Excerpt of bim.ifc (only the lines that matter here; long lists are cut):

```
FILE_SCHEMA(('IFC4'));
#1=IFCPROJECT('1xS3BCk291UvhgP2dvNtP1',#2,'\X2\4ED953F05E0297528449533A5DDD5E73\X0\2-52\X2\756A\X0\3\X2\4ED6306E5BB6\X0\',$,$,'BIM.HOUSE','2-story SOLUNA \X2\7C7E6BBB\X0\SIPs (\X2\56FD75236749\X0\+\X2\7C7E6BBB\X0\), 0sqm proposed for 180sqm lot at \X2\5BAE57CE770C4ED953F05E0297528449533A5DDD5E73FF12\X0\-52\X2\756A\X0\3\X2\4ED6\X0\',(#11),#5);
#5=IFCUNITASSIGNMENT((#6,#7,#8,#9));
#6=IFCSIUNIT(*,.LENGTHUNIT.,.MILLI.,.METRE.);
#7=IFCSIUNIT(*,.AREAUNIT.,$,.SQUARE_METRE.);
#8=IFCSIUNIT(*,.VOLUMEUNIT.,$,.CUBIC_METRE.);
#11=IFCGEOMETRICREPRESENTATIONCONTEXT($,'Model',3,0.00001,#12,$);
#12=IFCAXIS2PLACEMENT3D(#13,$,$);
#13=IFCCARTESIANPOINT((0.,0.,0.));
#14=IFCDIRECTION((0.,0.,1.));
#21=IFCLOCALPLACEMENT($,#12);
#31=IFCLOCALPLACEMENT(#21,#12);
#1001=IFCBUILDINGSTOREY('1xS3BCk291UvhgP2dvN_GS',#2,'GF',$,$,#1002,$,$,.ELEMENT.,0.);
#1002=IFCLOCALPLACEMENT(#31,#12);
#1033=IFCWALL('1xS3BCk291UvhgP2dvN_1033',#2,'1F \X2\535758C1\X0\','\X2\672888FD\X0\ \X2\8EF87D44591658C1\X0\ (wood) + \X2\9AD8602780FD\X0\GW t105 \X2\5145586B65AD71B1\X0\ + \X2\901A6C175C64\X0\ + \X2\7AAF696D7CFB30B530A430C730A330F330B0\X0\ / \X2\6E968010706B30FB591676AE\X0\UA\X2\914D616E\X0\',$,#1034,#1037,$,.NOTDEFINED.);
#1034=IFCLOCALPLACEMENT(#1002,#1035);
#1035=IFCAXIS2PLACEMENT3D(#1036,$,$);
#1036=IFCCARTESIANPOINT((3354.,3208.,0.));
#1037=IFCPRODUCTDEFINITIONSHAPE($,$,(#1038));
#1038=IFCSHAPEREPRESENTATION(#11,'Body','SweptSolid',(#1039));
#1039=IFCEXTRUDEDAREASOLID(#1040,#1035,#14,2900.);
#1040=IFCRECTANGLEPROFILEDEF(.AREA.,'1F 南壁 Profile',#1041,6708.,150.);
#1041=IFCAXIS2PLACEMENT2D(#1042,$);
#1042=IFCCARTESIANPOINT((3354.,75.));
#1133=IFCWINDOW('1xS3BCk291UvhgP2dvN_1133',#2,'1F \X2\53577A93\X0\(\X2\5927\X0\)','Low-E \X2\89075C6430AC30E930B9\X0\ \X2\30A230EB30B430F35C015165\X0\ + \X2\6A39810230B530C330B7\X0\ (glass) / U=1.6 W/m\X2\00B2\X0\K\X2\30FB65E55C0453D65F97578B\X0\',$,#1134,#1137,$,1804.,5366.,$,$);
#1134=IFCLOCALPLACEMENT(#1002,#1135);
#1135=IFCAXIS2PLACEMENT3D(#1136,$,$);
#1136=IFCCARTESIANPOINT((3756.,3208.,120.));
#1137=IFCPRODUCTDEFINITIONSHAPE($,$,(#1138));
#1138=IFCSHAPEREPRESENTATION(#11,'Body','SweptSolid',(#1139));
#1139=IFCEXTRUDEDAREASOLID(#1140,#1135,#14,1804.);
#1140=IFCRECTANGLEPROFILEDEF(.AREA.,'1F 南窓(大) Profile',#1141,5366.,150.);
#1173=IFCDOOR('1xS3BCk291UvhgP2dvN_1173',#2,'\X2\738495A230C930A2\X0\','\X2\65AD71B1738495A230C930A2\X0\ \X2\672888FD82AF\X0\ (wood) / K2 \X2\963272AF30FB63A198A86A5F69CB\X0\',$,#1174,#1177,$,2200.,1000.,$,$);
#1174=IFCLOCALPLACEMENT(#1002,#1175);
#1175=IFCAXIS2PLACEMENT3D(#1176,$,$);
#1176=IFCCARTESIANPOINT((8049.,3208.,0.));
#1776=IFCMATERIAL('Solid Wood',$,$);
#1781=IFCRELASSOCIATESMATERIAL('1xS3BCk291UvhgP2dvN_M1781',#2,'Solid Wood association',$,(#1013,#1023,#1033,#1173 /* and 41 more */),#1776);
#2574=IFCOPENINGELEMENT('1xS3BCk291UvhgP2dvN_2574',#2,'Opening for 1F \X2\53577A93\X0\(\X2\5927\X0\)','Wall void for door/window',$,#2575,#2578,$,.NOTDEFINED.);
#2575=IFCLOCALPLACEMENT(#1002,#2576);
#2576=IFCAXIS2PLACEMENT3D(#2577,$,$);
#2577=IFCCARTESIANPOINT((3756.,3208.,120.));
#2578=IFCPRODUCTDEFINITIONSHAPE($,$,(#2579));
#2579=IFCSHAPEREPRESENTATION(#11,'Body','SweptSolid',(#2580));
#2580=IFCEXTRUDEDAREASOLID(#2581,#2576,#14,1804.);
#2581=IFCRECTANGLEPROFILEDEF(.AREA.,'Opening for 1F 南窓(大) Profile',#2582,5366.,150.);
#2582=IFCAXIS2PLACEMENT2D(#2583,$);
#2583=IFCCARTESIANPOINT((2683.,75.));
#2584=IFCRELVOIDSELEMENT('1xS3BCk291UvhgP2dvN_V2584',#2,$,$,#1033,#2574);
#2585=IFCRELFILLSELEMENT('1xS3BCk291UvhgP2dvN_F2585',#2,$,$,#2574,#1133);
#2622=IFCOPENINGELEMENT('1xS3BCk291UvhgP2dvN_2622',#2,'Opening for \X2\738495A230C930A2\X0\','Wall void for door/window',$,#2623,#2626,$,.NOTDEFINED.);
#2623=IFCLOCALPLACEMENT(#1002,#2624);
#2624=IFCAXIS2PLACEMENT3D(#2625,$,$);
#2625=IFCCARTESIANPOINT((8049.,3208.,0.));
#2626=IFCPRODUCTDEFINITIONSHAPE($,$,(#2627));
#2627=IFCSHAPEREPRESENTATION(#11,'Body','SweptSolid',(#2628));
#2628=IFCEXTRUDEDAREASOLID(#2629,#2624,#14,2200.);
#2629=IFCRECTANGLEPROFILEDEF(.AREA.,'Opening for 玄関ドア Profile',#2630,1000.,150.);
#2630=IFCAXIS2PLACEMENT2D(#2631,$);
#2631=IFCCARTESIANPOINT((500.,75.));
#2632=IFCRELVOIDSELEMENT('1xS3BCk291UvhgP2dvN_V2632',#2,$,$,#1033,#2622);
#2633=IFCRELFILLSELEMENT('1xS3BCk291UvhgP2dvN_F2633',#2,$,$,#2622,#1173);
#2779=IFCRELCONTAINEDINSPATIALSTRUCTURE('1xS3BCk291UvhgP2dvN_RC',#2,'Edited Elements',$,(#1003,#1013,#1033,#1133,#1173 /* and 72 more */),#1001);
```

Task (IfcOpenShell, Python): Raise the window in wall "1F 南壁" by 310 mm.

```python
import numpy as np
import ifcopenshell
import ifcopenshell.api.geometry
import ifcopenshell.util.placement
import ifcopenshell.util.unit

model = ifcopenshell.open("bim.ifc")
unit_scale = ifcopenshell.util.unit.calculate_unit_scale(model)

window = model.by_guid("1xS3BCk291UvhgP2dvN_1133")
opening = window.FillsVoids[0].RelatingOpeningElement
dz = 310.0

shift = np.array([0.0, 0.0, dz])
# The window is not placed relative to its opening, so move both.
for product in (opening, window):
    matrix = ifcopenshell.util.placement.get_local_placement(product.ObjectPlacement)
    matrix[:3, 3] += shift
    ifcopenshell.api.geometry.edit_object_placement(model, product=product, matrix=matrix, is_si=False)

print(f"moved by {dz * unit_scale:+.3f} m")

model.write("bim_rev.ifc")
```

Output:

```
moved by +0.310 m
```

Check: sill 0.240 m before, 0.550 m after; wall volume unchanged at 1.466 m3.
